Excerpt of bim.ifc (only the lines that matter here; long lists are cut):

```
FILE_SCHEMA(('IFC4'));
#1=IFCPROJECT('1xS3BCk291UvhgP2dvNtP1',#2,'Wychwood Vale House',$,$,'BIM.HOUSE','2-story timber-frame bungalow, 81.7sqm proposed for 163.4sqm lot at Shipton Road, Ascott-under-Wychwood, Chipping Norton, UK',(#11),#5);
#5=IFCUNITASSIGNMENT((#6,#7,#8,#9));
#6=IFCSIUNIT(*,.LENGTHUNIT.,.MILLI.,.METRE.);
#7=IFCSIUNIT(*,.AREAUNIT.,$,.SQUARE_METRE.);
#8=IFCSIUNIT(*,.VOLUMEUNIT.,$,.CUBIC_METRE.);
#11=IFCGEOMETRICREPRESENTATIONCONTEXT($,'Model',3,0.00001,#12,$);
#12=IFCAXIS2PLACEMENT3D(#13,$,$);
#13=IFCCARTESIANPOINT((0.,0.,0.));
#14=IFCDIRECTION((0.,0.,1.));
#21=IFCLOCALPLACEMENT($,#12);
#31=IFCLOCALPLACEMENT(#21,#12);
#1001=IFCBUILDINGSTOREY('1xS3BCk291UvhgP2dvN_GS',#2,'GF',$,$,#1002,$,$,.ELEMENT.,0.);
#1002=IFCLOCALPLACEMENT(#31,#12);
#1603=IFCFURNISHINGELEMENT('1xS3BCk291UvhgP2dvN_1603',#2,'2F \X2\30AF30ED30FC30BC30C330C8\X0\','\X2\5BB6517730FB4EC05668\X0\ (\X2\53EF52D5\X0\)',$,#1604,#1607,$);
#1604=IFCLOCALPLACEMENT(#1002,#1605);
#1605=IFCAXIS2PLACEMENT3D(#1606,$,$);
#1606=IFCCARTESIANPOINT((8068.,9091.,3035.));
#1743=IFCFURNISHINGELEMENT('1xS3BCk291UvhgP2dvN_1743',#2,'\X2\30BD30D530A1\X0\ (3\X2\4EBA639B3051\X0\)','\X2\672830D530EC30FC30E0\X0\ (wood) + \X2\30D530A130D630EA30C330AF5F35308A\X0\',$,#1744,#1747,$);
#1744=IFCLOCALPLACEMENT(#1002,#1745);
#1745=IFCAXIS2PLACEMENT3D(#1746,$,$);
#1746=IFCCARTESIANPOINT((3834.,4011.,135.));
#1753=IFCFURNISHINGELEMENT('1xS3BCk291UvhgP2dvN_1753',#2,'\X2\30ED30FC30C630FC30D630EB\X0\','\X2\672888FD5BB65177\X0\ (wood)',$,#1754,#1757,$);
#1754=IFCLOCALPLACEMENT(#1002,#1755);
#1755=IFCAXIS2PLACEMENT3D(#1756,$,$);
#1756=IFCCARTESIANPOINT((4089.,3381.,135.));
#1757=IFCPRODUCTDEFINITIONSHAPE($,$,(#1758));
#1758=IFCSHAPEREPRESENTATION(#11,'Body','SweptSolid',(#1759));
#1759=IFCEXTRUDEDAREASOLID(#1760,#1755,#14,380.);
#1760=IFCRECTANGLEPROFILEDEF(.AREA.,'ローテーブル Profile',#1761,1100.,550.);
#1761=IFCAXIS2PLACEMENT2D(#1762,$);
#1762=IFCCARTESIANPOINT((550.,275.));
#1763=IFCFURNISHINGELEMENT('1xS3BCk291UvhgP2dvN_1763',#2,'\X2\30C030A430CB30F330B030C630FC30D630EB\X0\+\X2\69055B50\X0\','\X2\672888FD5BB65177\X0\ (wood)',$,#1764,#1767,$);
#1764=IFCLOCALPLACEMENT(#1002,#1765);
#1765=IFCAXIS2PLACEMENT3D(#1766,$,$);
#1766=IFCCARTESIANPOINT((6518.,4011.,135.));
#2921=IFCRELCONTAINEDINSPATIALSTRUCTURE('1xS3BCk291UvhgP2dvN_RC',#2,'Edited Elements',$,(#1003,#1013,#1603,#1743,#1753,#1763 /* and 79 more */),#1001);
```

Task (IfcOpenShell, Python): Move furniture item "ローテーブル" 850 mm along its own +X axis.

```python
import ifcopenshell
import ifcopenshell.api.geometry
import ifcopenshell.util.placement

model = ifcopenshell.open("bim.ifc")

item = model.by_guid("1xS3BCk291UvhgP2dvN_1753")
matrix = ifcopenshell.util.placement.get_local_placement(item.ObjectPlacement)
matrix[:3, 3] += matrix[:3, 0] * 850.0
ifcopenshell.api.geometry.edit_object_placement(model, product=item, matrix=matrix, is_si=False)

print(ifcopenshell.util.placement.get_local_placement(item.ObjectPlacement).round(3) + 0.0)

model.write("bim_edited.ifc")
```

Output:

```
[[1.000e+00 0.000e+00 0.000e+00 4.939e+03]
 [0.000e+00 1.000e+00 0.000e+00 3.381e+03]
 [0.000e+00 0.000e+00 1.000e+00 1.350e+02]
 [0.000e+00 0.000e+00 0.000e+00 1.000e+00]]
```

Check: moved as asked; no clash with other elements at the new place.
